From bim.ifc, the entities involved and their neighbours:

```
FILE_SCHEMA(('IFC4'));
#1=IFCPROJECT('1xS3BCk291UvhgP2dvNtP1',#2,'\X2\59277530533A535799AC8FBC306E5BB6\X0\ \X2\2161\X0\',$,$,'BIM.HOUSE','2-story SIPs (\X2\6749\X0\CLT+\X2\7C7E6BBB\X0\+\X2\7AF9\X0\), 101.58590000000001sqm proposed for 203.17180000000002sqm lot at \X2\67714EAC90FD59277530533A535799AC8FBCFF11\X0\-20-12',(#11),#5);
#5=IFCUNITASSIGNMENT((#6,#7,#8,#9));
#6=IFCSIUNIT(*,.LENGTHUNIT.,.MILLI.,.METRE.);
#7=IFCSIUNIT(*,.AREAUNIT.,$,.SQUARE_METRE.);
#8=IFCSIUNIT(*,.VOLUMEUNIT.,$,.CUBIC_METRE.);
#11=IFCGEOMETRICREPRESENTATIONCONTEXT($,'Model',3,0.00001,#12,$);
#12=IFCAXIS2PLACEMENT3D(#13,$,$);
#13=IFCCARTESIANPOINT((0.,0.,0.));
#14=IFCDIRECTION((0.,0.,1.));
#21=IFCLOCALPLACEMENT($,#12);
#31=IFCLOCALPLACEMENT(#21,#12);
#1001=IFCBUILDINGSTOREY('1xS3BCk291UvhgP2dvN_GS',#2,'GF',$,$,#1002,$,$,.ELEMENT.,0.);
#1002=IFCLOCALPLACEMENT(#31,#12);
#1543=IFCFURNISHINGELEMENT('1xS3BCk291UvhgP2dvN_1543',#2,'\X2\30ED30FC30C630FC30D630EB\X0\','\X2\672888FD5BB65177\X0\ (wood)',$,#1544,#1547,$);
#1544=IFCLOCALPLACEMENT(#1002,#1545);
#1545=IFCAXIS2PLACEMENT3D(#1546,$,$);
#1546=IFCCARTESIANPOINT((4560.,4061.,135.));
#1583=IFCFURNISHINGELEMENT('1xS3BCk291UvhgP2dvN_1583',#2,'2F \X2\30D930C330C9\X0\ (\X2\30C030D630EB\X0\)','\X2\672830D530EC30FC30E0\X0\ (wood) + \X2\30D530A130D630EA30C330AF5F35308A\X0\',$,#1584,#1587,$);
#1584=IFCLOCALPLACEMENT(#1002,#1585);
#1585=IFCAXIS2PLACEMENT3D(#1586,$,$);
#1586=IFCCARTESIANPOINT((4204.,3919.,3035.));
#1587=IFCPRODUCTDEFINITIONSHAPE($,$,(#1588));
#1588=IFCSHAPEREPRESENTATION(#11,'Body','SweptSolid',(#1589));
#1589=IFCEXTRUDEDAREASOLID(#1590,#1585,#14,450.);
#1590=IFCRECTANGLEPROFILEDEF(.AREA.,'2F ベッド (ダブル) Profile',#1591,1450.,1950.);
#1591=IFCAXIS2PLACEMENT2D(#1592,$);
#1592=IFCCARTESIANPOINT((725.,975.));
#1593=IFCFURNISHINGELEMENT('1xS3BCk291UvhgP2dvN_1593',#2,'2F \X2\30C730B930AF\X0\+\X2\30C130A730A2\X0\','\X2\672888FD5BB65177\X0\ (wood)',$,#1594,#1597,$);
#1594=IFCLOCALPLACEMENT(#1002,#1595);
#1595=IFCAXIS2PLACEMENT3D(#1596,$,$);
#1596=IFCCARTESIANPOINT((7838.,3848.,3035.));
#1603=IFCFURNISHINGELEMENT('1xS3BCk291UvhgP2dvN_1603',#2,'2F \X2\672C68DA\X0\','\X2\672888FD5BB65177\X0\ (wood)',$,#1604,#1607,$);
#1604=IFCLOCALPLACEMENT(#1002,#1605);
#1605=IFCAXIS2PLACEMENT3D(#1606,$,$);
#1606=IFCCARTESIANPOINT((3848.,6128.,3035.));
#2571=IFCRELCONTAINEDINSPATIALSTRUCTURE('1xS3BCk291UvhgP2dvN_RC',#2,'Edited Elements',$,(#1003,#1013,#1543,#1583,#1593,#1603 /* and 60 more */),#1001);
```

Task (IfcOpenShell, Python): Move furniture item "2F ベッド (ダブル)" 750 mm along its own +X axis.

```python
import ifcopenshell
import ifcopenshell.api.geometry
import ifcopenshell.util.placement

model = ifcopenshell.open("bim.ifc")

item = model.by_guid("1xS3BCk291UvhgP2dvN_1583")
matrix = ifcopenshell.util.placement.get_local_placement(item.ObjectPlacement)
matrix[:3, 3] += matrix[:3, 0] * 750.0
ifcopenshell.api.geometry.edit_object_placement(model, product=item, matrix=matrix, is_si=False)

print(ifcopenshell.util.placement.get_local_placement(item.ObjectPlacement).round(3) + 0.0)

model.write("bim_updated.ifc")
```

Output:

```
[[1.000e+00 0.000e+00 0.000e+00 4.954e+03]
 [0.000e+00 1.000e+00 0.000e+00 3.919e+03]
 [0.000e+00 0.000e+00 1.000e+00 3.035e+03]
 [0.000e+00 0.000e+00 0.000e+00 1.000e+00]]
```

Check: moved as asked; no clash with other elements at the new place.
